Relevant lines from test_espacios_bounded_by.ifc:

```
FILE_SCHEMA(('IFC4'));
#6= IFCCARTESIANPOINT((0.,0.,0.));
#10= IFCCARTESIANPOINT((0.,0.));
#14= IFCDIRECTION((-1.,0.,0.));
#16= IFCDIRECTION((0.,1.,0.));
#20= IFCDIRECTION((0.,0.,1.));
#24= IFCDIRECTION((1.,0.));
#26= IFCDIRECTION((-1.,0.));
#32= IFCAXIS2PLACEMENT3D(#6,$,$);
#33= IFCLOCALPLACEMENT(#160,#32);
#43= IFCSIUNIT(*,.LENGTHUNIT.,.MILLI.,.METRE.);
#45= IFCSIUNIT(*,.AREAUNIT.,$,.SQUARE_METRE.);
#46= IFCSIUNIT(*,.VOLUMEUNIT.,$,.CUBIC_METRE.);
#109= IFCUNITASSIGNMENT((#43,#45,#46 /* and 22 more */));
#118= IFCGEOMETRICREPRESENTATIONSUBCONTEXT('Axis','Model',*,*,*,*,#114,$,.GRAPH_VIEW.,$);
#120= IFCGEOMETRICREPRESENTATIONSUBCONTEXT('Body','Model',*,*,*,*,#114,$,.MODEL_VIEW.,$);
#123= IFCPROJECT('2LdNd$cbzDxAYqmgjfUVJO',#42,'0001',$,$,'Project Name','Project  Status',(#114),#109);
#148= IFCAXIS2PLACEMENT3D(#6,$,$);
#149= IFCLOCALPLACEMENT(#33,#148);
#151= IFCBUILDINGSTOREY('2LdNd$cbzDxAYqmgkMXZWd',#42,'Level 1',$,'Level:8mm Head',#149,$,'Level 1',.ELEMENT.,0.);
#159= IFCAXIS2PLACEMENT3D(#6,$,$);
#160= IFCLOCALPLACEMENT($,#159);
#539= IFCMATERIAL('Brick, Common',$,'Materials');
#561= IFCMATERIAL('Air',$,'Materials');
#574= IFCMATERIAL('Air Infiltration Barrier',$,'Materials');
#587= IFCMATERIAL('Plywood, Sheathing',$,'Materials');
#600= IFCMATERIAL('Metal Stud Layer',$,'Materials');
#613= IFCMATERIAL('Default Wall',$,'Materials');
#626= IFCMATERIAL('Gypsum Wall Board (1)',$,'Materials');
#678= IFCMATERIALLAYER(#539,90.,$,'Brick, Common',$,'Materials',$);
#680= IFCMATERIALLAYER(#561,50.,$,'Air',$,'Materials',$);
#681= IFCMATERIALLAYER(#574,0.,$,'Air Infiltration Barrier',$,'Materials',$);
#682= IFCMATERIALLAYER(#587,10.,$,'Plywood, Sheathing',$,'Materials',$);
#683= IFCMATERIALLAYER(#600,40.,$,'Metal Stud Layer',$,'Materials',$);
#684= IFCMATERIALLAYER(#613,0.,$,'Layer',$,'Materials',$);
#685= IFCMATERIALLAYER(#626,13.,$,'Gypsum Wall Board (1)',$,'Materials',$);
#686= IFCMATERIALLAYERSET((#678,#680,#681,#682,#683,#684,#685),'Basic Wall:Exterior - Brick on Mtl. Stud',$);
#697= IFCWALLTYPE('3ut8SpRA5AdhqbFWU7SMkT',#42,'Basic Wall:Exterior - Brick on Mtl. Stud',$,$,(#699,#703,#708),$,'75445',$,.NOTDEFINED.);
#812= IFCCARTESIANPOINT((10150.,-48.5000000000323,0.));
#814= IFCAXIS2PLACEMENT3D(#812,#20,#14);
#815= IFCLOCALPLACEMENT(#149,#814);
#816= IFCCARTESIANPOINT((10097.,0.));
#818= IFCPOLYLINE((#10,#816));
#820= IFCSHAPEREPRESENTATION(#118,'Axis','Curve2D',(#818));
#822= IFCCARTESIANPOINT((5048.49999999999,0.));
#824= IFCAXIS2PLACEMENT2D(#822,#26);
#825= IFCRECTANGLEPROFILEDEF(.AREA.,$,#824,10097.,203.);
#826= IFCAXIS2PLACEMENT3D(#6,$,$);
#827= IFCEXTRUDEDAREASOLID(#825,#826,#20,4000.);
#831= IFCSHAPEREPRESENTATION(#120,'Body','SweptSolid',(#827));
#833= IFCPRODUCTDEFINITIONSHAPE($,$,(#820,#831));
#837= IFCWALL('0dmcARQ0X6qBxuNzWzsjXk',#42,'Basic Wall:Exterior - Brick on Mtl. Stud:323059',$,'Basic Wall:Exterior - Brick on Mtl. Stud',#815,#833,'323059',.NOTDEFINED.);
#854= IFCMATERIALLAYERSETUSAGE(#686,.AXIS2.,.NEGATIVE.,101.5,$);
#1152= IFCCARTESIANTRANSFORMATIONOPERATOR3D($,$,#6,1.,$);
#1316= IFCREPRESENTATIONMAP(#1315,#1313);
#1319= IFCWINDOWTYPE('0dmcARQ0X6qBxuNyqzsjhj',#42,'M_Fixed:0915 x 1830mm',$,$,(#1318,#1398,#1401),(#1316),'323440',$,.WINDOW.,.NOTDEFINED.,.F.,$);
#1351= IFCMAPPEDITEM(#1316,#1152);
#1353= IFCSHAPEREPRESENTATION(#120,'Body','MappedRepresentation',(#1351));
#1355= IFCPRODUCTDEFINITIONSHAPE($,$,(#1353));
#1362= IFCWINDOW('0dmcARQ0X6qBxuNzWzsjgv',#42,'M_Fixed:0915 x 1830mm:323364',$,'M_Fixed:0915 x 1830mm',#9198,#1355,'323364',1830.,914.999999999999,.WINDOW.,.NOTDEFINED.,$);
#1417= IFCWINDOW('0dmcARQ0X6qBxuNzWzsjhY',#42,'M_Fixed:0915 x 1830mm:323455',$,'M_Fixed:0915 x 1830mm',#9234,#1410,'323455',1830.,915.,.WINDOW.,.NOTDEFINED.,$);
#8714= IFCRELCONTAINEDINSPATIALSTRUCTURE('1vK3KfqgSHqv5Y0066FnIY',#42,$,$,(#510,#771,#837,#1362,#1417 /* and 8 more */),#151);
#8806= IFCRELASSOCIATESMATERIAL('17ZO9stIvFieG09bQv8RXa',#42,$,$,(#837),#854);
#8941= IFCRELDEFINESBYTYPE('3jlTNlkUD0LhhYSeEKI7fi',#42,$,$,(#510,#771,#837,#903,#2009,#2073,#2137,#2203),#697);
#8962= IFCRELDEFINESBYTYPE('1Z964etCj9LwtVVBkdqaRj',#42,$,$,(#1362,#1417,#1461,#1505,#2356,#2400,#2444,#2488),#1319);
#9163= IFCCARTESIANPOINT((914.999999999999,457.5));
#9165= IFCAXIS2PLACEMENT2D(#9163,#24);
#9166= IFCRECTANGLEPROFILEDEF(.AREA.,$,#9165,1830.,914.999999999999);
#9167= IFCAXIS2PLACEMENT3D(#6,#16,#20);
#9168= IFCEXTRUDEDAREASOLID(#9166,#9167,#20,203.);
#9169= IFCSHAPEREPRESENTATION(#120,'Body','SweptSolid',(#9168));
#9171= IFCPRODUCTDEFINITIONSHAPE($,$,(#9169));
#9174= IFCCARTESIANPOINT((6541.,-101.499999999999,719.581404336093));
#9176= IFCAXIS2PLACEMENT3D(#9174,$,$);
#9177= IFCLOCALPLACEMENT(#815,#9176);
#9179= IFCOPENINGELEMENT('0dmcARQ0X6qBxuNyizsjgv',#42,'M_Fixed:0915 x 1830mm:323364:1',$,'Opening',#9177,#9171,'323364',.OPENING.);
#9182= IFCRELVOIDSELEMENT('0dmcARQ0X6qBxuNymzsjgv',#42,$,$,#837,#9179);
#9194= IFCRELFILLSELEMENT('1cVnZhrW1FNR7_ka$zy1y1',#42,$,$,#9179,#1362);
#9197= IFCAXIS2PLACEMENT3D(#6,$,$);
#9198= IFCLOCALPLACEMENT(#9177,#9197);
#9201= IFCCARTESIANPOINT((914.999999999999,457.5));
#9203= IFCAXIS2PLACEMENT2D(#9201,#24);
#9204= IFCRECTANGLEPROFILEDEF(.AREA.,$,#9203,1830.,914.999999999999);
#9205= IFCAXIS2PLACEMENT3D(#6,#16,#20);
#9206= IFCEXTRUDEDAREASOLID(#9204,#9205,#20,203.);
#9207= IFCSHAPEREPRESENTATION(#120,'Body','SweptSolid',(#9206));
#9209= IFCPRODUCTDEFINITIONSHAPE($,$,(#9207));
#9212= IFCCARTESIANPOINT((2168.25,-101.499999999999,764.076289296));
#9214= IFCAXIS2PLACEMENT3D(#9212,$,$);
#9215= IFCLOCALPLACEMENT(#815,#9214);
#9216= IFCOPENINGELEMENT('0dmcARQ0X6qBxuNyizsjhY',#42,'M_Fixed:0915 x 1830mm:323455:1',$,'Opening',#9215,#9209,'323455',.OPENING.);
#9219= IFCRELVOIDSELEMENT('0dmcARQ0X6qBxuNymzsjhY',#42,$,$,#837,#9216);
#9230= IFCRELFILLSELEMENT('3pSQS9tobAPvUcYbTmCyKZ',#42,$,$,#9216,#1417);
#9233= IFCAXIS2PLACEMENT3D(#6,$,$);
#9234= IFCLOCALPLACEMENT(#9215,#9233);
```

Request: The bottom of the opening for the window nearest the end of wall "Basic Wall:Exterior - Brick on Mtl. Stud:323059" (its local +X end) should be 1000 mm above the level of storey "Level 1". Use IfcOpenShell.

```python
import numpy as np
import ifcopenshell
import ifcopenshell.api.geometry
import ifcopenshell.geom
import ifcopenshell.util.element
import ifcopenshell.util.placement
import ifcopenshell.util.shape
import ifcopenshell.util.unit

model = ifcopenshell.open("test_espacios_bounded_by.ifc")
unit_scale = ifcopenshell.util.unit.calculate_unit_scale(model)

window = model.by_id(1362)
opening = window.FillsVoids[0].RelatingOpeningElement
storey = ifcopenshell.util.element.get_container(window, ifc_class="IfcBuildingStorey")
level = ifcopenshell.util.placement.get_local_placement(storey.ObjectPlacement)[2, 3]

# The opening's origin need not be at the sill, so measure its lowest point.
shape = ifcopenshell.geom.create_shape(ifcopenshell.geom.settings(), opening)
bottom = ifcopenshell.util.shape.get_shape_bottom_elevation(shape, shape.geometry) / unit_scale
dz = level + 1 / unit_scale - bottom

shift = np.array([0.0, 0.0, dz])
# The window is placed relative to its opening, so it follows when the opening moves.
matrix = ifcopenshell.util.placement.get_local_placement(opening.ObjectPlacement)
matrix[:3, 3] += shift
ifcopenshell.api.geometry.edit_object_placement(
    model, product=opening, matrix=matrix, is_si=False, should_transform_children=True
)

print(f"moved by {dz * unit_scale:+.3f} m")

model.write("test_espacios_bounded_by_rev.ifc")
```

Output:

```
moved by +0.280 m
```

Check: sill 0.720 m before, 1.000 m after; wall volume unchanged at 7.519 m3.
